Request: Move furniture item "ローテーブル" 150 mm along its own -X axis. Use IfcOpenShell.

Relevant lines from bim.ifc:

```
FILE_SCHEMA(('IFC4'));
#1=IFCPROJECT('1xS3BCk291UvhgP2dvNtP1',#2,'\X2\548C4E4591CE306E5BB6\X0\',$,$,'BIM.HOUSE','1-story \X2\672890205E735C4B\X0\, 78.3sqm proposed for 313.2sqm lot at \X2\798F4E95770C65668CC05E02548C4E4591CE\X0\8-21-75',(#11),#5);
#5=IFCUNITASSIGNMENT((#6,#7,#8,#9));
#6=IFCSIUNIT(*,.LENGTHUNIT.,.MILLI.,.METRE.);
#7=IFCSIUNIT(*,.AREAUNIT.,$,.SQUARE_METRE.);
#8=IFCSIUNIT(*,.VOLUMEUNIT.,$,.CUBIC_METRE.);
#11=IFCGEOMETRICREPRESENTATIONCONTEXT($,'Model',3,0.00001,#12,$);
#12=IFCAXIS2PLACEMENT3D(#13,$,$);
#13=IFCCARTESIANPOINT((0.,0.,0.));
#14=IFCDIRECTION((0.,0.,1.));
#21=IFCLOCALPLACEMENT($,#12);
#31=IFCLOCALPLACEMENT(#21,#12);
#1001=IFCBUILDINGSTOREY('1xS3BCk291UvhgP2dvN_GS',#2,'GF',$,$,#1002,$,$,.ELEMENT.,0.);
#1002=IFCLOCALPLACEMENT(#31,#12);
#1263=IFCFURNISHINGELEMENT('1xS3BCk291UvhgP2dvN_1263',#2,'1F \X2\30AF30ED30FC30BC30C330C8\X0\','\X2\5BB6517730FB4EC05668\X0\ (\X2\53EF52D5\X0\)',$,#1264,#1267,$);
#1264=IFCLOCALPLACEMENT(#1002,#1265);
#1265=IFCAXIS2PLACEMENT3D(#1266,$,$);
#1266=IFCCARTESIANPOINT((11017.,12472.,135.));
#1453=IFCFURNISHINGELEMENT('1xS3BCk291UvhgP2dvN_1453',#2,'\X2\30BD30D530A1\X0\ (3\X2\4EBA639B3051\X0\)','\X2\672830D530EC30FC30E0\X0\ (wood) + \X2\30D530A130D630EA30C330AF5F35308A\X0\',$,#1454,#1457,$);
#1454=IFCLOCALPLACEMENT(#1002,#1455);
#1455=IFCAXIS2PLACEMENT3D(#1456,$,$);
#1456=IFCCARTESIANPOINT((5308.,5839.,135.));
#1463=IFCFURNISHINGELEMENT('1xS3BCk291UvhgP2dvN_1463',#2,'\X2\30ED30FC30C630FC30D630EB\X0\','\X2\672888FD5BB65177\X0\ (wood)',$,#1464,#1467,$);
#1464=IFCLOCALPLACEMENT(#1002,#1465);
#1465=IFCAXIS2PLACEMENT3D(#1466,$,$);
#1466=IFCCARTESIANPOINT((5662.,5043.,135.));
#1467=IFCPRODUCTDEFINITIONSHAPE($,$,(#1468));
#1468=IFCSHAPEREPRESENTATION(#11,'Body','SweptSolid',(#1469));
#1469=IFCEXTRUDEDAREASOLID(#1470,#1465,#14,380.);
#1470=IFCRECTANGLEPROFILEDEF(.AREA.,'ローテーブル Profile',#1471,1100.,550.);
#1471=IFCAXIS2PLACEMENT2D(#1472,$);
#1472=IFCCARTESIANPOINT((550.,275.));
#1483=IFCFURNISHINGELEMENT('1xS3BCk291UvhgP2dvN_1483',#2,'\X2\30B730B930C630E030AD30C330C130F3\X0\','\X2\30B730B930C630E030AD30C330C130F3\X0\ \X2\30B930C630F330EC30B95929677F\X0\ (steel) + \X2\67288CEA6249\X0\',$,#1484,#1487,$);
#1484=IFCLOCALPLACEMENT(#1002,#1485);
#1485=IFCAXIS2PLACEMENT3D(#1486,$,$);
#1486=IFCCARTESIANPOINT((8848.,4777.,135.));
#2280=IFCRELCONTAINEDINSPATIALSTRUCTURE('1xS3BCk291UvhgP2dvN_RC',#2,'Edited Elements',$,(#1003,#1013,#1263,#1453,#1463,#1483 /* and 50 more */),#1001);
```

```python
import ifcopenshell
import ifcopenshell.api.geometry
import ifcopenshell.util.placement

model = ifcopenshell.open("bim.ifc")

item = model.by_guid("1xS3BCk291UvhgP2dvN_1463")
matrix = ifcopenshell.util.placement.get_local_placement(item.ObjectPlacement)
matrix[:3, 3] -= matrix[:3, 0] * 150.0
ifcopenshell.api.geometry.edit_object_placement(model, product=item, matrix=matrix, is_si=False)

print(ifcopenshell.util.placement.get_local_placement(item.ObjectPlacement).round(3) + 0.0)

model.write("bim-out.ifc")
```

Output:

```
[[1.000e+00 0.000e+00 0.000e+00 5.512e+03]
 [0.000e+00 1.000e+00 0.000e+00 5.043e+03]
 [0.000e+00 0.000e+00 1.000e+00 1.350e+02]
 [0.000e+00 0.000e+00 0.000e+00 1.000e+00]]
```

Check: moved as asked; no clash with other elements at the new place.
